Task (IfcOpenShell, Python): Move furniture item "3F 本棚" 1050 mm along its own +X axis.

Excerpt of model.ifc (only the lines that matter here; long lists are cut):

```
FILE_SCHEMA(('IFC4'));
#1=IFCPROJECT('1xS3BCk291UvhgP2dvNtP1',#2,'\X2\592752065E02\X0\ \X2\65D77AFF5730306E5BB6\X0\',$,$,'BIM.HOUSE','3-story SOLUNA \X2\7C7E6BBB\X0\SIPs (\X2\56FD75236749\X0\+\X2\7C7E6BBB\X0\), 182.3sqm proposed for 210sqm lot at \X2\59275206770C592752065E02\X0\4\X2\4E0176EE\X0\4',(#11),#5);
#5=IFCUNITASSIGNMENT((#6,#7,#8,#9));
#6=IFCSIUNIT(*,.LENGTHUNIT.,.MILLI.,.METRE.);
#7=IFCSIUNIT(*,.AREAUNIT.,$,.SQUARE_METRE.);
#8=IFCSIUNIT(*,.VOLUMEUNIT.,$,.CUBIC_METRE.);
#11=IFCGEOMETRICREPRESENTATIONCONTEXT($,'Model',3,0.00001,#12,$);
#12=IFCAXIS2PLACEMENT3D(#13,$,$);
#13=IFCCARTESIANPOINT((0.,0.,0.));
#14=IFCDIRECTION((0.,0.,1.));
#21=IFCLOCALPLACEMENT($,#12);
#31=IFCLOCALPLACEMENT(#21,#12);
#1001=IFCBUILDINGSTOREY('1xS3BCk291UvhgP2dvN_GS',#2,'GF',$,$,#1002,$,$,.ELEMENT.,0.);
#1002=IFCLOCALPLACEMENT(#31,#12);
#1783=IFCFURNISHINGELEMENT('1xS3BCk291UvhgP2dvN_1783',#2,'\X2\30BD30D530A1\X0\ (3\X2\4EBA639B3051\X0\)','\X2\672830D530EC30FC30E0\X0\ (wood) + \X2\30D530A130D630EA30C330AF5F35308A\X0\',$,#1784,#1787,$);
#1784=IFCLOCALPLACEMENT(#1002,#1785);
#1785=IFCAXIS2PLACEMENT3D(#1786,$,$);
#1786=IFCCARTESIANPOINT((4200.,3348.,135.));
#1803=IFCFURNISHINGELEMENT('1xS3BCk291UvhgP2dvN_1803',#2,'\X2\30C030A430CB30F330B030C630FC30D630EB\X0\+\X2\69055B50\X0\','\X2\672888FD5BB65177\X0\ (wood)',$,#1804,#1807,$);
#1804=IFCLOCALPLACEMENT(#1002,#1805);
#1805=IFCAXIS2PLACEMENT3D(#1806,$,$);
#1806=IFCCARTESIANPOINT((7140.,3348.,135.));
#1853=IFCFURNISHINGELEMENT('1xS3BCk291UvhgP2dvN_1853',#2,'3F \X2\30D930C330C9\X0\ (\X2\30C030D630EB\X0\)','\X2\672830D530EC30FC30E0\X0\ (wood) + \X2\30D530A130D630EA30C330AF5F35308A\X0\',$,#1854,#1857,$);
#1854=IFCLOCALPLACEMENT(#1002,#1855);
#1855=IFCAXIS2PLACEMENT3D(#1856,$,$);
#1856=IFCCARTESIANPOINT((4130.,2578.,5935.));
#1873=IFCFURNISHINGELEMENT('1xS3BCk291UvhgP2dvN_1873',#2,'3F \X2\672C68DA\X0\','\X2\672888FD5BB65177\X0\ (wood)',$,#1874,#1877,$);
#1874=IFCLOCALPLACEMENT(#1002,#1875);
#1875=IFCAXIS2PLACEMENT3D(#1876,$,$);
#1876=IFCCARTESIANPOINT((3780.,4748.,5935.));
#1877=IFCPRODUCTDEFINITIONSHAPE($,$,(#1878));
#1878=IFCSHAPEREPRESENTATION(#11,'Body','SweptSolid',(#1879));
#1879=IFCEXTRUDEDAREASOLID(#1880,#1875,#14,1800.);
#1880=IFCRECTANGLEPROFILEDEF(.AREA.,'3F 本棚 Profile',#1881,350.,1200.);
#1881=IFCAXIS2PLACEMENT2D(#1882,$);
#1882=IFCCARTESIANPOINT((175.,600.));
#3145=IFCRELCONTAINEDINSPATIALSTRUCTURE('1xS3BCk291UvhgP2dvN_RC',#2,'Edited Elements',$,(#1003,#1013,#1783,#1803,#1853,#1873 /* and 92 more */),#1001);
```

```python
import ifcopenshell
import ifcopenshell.api.geometry
import ifcopenshell.util.placement

model = ifcopenshell.open("model.ifc")

item = model.by_guid("1xS3BCk291UvhgP2dvN_1873")
matrix = ifcopenshell.util.placement.get_local_placement(item.ObjectPlacement)
matrix[:3, 3] += matrix[:3, 0] * 1050.0
ifcopenshell.api.geometry.edit_object_placement(model, product=item, matrix=matrix, is_si=False)

print(ifcopenshell.util.placement.get_local_placement(item.ObjectPlacement).round(3) + 0.0)

model.write("model_v2.ifc")
```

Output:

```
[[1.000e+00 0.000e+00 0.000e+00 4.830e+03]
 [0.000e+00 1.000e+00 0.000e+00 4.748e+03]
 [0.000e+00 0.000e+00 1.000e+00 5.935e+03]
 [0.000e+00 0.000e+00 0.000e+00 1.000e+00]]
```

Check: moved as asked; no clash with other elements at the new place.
